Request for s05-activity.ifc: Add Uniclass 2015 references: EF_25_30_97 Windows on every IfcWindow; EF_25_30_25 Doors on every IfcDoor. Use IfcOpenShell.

First a look at what the model holds.

```python
import ifcopenshell

model = ifcopenshell.open("s05-activity.ifc")
print(model.schema)
print("classifications:", [c.Name for c in model.by_type("IfcClassification")])
for ifc_class in ("IfcDoor", "IfcRoof", "IfcStair", "IfcWall", "IfcWindow"):
    print(ifc_class, len(model.by_type(ifc_class)))
```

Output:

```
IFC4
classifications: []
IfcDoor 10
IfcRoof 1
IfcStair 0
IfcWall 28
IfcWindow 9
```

```python
import ifcopenshell
import ifcopenshell.api.classification

model = ifcopenshell.open("s05-activity.ifc")

system = ifcopenshell.api.classification.add_classification(model, classification="Uniclass 2015")

codes = {
    "IfcWindow": ("EF_25_30_97", "Windows"),
    "IfcDoor": ("EF_25_30_25", "Doors"),
}
for ifc_class, (code, name) in codes.items():
    products = model.by_type(ifc_class)
    ifcopenshell.api.classification.add_reference(
        model, products=products, classification=system, identification=code, name=name
    )
    print(code, len(products))

model.write("s05-activity_v2.ifc")
```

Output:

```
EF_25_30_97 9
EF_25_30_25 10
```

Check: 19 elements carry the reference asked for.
